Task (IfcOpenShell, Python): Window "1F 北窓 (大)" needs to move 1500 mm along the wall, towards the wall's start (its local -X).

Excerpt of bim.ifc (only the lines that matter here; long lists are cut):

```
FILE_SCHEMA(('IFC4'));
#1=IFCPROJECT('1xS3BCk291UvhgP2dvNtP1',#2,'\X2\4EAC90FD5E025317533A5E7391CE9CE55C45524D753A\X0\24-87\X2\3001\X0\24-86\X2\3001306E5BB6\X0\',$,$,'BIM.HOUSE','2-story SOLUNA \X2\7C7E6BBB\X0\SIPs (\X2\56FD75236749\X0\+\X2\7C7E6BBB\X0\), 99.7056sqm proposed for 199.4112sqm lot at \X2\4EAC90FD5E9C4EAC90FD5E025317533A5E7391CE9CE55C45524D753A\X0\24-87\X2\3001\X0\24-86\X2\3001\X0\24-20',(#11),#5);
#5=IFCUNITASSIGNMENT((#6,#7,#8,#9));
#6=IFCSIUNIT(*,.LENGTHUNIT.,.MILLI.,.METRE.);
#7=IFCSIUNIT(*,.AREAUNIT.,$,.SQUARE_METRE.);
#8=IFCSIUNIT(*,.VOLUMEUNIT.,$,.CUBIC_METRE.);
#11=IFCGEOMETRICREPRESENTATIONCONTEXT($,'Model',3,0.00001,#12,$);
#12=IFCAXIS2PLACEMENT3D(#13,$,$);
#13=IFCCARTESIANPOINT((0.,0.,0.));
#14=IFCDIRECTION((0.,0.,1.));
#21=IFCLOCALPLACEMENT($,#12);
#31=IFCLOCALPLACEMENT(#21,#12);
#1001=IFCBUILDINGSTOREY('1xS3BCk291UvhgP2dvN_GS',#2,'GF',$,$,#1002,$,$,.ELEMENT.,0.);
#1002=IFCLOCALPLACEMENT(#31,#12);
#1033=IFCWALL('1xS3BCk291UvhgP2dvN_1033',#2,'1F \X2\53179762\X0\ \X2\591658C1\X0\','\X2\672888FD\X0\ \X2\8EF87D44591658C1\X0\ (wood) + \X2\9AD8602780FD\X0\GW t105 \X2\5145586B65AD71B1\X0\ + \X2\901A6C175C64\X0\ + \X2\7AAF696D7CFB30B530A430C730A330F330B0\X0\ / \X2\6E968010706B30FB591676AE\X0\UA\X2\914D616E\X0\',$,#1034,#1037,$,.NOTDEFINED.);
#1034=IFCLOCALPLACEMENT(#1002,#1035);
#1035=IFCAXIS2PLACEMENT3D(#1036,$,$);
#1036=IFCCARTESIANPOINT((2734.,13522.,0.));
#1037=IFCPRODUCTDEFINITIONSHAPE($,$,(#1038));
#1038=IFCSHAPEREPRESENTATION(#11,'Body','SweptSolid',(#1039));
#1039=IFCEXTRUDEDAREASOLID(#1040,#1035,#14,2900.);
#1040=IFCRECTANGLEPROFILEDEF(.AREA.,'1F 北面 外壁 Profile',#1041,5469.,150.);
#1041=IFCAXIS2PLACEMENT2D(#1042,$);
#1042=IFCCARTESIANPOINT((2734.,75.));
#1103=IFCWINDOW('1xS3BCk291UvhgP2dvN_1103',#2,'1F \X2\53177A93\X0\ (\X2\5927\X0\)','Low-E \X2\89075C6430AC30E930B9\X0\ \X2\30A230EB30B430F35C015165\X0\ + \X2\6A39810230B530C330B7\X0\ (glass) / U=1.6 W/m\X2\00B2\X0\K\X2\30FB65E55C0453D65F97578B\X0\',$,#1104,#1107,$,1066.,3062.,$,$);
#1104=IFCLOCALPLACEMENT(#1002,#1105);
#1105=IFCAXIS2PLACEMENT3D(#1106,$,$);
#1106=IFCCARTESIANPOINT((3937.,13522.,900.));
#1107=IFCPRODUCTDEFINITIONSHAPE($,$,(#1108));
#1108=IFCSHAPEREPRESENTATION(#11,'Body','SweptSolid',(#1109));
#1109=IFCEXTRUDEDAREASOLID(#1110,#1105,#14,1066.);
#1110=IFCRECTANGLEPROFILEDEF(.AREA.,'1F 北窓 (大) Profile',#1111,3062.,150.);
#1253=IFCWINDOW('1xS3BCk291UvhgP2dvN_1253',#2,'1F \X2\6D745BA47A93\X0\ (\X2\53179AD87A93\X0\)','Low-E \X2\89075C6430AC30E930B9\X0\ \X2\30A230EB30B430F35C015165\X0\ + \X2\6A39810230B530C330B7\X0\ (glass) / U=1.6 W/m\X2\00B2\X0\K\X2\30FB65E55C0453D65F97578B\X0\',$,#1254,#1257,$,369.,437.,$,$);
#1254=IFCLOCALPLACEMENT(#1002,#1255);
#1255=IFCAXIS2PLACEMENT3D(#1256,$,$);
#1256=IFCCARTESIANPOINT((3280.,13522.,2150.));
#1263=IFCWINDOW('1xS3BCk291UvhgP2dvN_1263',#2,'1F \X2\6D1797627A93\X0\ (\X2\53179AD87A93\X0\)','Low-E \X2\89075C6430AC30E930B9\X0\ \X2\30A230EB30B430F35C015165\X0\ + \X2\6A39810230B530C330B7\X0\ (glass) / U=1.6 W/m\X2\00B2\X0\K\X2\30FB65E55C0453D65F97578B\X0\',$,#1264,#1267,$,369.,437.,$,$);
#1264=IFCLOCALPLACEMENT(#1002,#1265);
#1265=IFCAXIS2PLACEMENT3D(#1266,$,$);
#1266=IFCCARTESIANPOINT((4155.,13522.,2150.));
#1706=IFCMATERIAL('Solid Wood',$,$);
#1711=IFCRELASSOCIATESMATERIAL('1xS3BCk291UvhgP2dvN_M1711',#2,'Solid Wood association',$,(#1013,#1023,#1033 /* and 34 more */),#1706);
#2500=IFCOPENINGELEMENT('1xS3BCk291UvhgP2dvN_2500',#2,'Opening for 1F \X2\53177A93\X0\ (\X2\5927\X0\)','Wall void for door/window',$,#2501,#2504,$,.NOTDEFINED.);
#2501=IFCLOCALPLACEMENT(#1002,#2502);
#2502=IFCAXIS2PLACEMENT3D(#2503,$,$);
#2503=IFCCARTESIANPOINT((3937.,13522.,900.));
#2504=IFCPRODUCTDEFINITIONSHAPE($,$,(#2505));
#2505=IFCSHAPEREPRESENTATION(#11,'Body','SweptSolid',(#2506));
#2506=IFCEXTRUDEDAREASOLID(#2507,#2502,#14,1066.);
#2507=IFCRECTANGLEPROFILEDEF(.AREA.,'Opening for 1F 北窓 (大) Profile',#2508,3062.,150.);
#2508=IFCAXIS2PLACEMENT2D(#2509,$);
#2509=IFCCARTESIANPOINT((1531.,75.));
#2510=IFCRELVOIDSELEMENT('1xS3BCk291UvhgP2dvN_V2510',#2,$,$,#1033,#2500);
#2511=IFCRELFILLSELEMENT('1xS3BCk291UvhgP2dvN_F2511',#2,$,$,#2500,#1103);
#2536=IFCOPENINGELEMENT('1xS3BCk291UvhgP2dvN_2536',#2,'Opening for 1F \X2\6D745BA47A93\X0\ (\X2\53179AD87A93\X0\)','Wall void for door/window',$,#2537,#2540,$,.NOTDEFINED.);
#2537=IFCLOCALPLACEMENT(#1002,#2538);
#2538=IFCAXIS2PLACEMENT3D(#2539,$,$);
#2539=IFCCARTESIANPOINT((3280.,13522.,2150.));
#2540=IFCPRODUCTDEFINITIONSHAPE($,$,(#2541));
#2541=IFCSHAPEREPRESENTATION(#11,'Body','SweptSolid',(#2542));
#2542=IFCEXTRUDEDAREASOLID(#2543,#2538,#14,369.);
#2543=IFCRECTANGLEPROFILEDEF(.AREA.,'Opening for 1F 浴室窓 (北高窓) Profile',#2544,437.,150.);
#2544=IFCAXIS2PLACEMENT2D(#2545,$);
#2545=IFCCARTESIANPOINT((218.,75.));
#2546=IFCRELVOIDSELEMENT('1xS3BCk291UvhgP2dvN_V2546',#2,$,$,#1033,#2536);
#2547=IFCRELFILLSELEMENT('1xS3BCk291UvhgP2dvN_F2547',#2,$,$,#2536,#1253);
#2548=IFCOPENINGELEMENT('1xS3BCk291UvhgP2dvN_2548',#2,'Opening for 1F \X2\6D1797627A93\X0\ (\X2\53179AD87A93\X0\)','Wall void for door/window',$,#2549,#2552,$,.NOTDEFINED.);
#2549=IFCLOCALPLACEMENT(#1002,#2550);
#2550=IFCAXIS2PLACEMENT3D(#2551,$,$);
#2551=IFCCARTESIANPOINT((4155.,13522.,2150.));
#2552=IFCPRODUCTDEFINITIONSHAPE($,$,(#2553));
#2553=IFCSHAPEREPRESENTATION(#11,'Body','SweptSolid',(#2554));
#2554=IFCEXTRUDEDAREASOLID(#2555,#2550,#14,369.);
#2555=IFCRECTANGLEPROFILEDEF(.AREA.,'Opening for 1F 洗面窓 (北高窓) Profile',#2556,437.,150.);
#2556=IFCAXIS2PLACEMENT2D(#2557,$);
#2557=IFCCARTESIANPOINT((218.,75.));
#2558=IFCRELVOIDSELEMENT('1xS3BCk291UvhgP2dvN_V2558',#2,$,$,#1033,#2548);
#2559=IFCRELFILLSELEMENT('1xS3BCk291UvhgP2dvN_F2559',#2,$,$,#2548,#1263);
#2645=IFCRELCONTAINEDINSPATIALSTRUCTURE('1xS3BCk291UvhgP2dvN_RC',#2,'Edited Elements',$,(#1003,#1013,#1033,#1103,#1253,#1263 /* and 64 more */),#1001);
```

```python
import ifcopenshell
import ifcopenshell.api.geometry
import ifcopenshell.util.placement

model = ifcopenshell.open("bim.ifc")

window = model.by_guid("1xS3BCk291UvhgP2dvN_1103")
opening = window.FillsVoids[0].RelatingOpeningElement
wall = opening.VoidsElements[0].RelatingBuildingElement

wall_matrix = ifcopenshell.util.placement.get_local_placement(wall.ObjectPlacement)
shift = wall_matrix[:3, 0] * -1500.0
before = ifcopenshell.util.placement.get_local_placement(window.ObjectPlacement)[:3, 3].copy()

# The window is not placed relative to its opening, so move both.
for product in (opening, window):
    matrix = ifcopenshell.util.placement.get_local_placement(product.ObjectPlacement)
    matrix[:3, 3] += shift
    ifcopenshell.api.geometry.edit_object_placement(model, product=product, matrix=matrix, is_si=False)

after = ifcopenshell.util.placement.get_local_placement(window.ObjectPlacement)[:3, 3]
print("window moved by", (after - before).round(3) + 0.0)

model.write("bim_edited.ifc")
```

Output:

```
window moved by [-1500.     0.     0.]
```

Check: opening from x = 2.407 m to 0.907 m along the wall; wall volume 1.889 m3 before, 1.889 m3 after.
